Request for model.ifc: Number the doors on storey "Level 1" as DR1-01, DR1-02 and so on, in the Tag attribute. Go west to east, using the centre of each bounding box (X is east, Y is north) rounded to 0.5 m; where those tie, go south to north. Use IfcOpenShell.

First a look at what the model holds.

```python
import ifcopenshell
import ifcopenshell.util.element
import ifcopenshell.util.placement

model = ifcopenshell.open("model.ifc")
print(model.schema)
storey = next(s for s in model.by_type("IfcBuildingStorey") if s.Name == "Level 1")
doors = [e for e in ifcopenshell.util.element.get_decomposition(storey) if e.is_a("IfcDoor")]
for e in sorted(doors, key=lambda e: e.id()):
    origin = ifcopenshell.util.placement.get_local_placement(e.ObjectPlacement)[:3, 3]
    print(e.id(), e.Tag, e.Name, origin.round(2) + 0.0, sep=" | ")
```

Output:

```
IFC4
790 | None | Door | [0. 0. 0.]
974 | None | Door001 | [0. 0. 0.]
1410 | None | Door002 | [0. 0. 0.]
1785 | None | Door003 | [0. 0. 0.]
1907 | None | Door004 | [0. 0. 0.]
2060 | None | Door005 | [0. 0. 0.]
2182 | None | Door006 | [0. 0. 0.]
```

```python
import ifcopenshell
import ifcopenshell.geom
import ifcopenshell.util.element
import ifcopenshell.util.shape

model = ifcopenshell.open("model.ifc")
settings = ifcopenshell.geom.settings()
settings.set("use-world-coords", True)


def centre(element):
    shape = ifcopenshell.geom.create_shape(settings, element)
    return ifcopenshell.util.shape.get_bbox_centroid(shape.geometry)


storey = next(s for s in model.by_type("IfcBuildingStorey") if s.Name == "Level 1")
doors = [e for e in ifcopenshell.util.element.get_decomposition(storey) if e.is_a("IfcDoor")]

# Insertion points can sit at a corner or the storey origin, so sort by the geometry (in metres).
centres = {e: centre(e) for e in doors}
doors.sort(key=lambda e: (round(centres[e][0] / 0.5), centres[e][1]))

for i, e in enumerate(doors, start=1):
    number = f"DR1-{i:02d}"
    e.Tag = number
    print(e.id(), number)

model.write("model_v2.ifc")
```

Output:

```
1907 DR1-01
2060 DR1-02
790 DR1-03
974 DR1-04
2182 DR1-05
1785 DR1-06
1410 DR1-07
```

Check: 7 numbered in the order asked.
